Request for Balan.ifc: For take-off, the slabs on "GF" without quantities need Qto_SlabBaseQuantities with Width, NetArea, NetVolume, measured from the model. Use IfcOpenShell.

First a look at what the model holds.

```python
import ifcopenshell
import ifcopenshell.util.element
import ifcopenshell.util.unit

model = ifcopenshell.open("Balan.ifc")
print(model.schema)
for unit_type in ("LENGTHUNIT", "AREAUNIT", "VOLUMEUNIT"):
    print(unit_type, ifcopenshell.util.unit.calculate_unit_scale(model, unit_type))
storey = next(s for s in model.by_type("IfcBuildingStorey") if s.Name == "GF")
slabs = [e for e in ifcopenshell.util.element.get_decomposition(storey) if e.is_a("IfcSlab")]
for e in sorted(slabs, key=lambda e: e.id()):
    print(e.id(), e.is_a(), e.Name, list(ifcopenshell.util.element.get_psets(e, qtos_only=True)), sep=" | ")
```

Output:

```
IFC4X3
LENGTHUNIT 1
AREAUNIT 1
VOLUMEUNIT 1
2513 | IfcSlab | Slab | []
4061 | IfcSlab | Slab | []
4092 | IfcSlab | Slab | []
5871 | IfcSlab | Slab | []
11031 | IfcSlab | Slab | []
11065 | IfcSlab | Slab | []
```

```python
import ifcopenshell
import ifcopenshell.api.pset
import ifcopenshell.geom
import ifcopenshell.util.element
import ifcopenshell.util.shape
import ifcopenshell.util.unit

model = ifcopenshell.open("Balan.ifc")
unit_scale = ifcopenshell.util.unit.calculate_unit_scale(model)
area_scale = ifcopenshell.util.unit.calculate_unit_scale(model, "AREAUNIT")
volume_scale = ifcopenshell.util.unit.calculate_unit_scale(model, "VOLUMEUNIT")
settings = ifcopenshell.geom.settings()

storey = next(s for s in model.by_type("IfcBuildingStorey") if s.Name == "GF")
slabs = [e for e in ifcopenshell.util.element.get_decomposition(storey) if e.is_a("IfcSlab")]

for e in sorted(slabs, key=lambda e: e.id()):
    if ifcopenshell.util.element.get_psets(e, qtos_only=True, should_inherit=False):
        continue
    # Geometry comes back in metres, in the element's own axes.
    shape = ifcopenshell.geom.create_shape(settings, e)
    values = {
        "Width": ifcopenshell.util.shape.get_z(shape.geometry) / unit_scale,
        "NetArea": ifcopenshell.util.shape.get_footprint_area(shape.geometry) / area_scale,
        "NetVolume": ifcopenshell.util.shape.get_volume(shape.geometry) / volume_scale,
    }
    qto = ifcopenshell.api.pset.add_qto(model, product=e, name="Qto_SlabBaseQuantities")
    ifcopenshell.api.pset.edit_qto(model, qto=qto, properties=values)
    print(e.id(), {k: round(v, 3) for k, v in values.items()})

model.write("Balan-out.ifc")
```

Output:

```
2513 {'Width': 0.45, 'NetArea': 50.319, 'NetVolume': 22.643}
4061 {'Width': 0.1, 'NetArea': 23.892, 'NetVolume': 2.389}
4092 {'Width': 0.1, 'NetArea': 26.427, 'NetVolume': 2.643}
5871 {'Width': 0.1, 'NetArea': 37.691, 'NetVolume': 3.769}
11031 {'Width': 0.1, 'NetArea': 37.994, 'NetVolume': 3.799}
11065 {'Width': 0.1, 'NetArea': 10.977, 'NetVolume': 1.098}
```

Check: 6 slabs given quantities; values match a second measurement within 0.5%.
